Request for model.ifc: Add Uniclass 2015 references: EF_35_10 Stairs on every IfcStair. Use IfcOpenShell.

First a look at what the model holds.

```python
import ifcopenshell

model = ifcopenshell.open("model.ifc")
print(model.schema)
print("classifications:", [c.Name for c in model.by_type("IfcClassification")])
for ifc_class in ("IfcDoor", "IfcRoof", "IfcStair", "IfcWall", "IfcWindow"):
    print(ifc_class, len(model.by_type(ifc_class)))
```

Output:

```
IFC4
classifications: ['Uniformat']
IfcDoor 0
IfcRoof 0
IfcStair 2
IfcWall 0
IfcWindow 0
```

```python
import ifcopenshell
import ifcopenshell.api.classification

model = ifcopenshell.open("model.ifc")

system = ifcopenshell.api.classification.add_classification(model, classification="Uniclass 2015")

codes = {
    "IfcStair": ("EF_35_10", "Stairs"),
}
for ifc_class, (code, name) in codes.items():
    products = model.by_type(ifc_class)
    ifcopenshell.api.classification.add_reference(
        model, products=products, classification=system, identification=code, name=name
    )
    print(code, len(products))

model.write("model_updated.ifc")
```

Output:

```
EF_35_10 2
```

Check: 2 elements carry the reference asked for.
